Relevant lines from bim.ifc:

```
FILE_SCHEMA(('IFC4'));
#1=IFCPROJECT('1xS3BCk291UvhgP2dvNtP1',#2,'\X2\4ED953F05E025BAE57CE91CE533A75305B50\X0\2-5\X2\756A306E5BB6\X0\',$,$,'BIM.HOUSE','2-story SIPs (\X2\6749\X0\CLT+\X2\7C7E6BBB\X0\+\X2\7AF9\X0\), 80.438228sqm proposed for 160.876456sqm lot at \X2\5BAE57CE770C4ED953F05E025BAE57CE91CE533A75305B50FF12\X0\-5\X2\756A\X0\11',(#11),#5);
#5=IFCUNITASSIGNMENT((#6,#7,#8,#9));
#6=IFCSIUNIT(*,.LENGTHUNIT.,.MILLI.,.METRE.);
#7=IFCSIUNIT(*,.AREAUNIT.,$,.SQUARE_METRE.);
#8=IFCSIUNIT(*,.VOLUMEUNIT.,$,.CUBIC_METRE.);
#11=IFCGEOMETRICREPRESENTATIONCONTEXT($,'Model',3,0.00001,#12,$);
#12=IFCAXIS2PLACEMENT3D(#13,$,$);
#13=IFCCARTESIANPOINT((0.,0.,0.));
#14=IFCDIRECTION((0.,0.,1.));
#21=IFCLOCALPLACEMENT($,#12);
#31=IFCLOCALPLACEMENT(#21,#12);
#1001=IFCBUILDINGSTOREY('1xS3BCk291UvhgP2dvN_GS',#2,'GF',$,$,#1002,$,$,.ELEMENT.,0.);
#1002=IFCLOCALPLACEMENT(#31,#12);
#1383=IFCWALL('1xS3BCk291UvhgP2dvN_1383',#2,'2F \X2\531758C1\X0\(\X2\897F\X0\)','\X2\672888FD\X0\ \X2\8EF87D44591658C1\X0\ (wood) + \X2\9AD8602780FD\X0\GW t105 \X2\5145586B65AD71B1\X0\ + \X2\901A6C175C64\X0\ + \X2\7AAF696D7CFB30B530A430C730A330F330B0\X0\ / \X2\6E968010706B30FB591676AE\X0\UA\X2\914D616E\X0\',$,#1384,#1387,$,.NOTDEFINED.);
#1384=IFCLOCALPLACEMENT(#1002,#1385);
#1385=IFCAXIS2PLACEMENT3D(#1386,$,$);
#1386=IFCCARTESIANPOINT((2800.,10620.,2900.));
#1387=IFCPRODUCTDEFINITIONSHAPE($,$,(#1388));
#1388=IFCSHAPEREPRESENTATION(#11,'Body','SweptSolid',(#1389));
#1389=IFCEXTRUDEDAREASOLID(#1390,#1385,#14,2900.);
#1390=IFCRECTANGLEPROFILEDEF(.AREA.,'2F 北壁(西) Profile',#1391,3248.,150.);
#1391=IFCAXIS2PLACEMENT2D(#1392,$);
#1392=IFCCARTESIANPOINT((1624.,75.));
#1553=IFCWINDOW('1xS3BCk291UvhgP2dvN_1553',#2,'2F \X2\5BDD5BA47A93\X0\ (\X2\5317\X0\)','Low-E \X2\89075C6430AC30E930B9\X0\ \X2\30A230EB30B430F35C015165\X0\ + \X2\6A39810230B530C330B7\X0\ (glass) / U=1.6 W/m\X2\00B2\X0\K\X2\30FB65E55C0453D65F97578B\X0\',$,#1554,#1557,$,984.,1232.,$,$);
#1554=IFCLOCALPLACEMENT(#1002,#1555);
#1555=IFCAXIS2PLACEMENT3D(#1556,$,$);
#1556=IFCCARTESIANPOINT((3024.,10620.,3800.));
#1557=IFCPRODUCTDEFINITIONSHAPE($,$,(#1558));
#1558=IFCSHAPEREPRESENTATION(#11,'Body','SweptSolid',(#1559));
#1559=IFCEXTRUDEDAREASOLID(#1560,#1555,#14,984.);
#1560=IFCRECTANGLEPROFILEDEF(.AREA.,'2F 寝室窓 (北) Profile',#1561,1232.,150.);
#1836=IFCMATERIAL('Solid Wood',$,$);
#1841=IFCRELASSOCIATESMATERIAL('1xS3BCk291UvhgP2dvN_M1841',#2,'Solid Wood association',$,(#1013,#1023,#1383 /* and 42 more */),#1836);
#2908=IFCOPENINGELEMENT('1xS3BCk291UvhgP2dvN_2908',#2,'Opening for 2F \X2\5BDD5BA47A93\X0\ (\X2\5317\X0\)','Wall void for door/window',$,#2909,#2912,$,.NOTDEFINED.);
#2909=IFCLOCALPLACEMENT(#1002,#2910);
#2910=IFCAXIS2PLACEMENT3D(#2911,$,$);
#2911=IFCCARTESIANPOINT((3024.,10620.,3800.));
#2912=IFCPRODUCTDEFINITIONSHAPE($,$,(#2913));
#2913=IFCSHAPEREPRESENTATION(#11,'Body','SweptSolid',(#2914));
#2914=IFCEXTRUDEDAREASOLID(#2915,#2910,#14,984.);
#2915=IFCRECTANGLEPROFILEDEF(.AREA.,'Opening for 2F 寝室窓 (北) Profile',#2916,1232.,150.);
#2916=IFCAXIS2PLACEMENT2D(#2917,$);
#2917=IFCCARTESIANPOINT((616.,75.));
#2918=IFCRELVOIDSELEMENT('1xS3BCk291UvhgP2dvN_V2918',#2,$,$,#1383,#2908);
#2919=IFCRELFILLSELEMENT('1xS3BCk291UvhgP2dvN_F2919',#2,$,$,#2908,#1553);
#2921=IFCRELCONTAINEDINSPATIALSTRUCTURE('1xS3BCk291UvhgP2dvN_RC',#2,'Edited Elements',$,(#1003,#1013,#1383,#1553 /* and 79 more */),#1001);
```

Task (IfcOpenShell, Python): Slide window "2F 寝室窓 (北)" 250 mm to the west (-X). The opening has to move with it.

```python
import ifcopenshell
import ifcopenshell.api.geometry
import ifcopenshell.util.placement
import ifcopenshell.util.unit

model = ifcopenshell.open("bim.ifc")
unit_scale = ifcopenshell.util.unit.calculate_unit_scale(model)

window = model.by_guid("1xS3BCk291UvhgP2dvN_1553")
opening = window.FillsVoids[0].RelatingOpeningElement
wall = opening.VoidsElements[0].RelatingBuildingElement

wall_matrix = ifcopenshell.util.placement.get_local_placement(wall.ObjectPlacement)
shift = wall_matrix[:3, 0] * -0.25 / unit_scale
before = ifcopenshell.util.placement.get_local_placement(window.ObjectPlacement)[:3, 3].copy()

# The window is not placed relative to its opening, so move both.
for product in (opening, window):
    matrix = ifcopenshell.util.placement.get_local_placement(product.ObjectPlacement)
    matrix[:3, 3] += shift
    ifcopenshell.api.geometry.edit_object_placement(model, product=product, matrix=matrix, is_si=False)

after = ifcopenshell.util.placement.get_local_placement(window.ObjectPlacement)[:3, 3]
print("window moved by", (after - before).round(3) + 0.0)

model.write("bim_rev.ifc")
```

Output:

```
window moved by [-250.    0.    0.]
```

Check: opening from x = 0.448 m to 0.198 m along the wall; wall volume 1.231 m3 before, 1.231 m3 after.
